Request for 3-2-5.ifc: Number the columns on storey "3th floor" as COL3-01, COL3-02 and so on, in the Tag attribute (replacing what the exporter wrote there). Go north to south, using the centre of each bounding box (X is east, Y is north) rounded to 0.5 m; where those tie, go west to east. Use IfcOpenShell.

First a look at what the model holds.

```python
import ifcopenshell
import ifcopenshell.util.element
import ifcopenshell.util.placement

model = ifcopenshell.open("3-2-5.ifc")
print(model.schema)
storey = next(s for s in model.by_type("IfcBuildingStorey") if s.Name == "3th floor")
columns = [e for e in ifcopenshell.util.element.get_decomposition(storey) if e.is_a("IfcColumn")]
for e in sorted(columns, key=lambda e: e.id()):
    origin = ifcopenshell.util.placement.get_local_placement(e.ObjectPlacement)[:3, 3]
    print(e.id(), e.Tag, e.Name, origin.round(2) + 0.0, sep=" | ")
```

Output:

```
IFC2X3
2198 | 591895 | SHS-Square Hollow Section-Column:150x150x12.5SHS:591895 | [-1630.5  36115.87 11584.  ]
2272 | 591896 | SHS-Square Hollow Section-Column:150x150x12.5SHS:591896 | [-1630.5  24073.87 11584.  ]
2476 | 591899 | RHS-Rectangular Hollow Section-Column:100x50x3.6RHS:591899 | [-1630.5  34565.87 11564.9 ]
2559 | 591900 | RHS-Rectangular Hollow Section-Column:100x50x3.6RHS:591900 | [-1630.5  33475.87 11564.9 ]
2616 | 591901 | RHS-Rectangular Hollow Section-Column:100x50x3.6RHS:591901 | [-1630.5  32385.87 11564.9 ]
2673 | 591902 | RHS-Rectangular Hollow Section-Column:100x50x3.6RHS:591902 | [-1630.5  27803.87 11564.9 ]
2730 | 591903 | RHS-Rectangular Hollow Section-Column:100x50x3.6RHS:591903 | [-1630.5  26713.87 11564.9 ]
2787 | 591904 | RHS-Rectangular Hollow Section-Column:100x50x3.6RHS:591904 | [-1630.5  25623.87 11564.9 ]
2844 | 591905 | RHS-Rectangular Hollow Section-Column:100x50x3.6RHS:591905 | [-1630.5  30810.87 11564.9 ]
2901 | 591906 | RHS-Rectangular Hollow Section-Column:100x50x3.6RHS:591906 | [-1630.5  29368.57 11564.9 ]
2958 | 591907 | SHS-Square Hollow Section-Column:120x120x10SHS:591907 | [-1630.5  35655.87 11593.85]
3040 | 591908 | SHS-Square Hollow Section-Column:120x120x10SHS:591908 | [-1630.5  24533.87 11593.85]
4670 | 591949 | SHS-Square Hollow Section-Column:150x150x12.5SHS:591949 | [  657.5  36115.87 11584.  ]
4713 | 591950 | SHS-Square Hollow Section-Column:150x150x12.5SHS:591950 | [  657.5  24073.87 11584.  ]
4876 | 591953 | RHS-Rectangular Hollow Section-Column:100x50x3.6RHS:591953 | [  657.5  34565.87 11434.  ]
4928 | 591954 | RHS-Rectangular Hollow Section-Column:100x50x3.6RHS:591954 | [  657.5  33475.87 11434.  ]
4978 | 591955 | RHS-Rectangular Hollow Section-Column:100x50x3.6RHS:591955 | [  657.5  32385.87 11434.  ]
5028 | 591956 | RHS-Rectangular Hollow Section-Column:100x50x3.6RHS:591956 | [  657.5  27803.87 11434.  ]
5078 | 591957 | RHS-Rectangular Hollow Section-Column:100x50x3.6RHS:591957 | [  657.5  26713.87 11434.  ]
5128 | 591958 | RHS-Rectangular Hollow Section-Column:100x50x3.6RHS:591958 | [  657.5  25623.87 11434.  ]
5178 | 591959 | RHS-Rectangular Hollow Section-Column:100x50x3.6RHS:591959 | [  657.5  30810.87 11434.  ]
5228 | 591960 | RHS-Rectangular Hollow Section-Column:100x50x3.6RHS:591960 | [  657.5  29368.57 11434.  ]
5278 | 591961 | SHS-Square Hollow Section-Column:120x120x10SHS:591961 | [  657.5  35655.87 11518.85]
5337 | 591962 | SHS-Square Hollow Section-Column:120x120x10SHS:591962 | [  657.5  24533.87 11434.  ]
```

```python
import ifcopenshell
import ifcopenshell.geom
import ifcopenshell.util.element
import ifcopenshell.util.shape

model = ifcopenshell.open("3-2-5.ifc")
settings = ifcopenshell.geom.settings()
settings.set("use-world-coords", True)


def centre(element):
    shape = ifcopenshell.geom.create_shape(settings, element)
    return ifcopenshell.util.shape.get_bbox_centroid(shape.geometry)


storey = next(s for s in model.by_type("IfcBuildingStorey") if s.Name == "3th floor")
columns = [e for e in ifcopenshell.util.element.get_decomposition(storey) if e.is_a("IfcColumn")]

# Insertion points can sit at a corner or the storey origin, so sort by the geometry (in metres).
centres = {e: centre(e) for e in columns}
columns.sort(key=lambda e: (-round(centres[e][1] / 0.5), centres[e][0]))

for i, e in enumerate(columns, start=1):
    number = f"COL3-{i:02d}"
    e.Tag = number
    print(e.id(), number)

model.write("3-2-5-out.ifc")
```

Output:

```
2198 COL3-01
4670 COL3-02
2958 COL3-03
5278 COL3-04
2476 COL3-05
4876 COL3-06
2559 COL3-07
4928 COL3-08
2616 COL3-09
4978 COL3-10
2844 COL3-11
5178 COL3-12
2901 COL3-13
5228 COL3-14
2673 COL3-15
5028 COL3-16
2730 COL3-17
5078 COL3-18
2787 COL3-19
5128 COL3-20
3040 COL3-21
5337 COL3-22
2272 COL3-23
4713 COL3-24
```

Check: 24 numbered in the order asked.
